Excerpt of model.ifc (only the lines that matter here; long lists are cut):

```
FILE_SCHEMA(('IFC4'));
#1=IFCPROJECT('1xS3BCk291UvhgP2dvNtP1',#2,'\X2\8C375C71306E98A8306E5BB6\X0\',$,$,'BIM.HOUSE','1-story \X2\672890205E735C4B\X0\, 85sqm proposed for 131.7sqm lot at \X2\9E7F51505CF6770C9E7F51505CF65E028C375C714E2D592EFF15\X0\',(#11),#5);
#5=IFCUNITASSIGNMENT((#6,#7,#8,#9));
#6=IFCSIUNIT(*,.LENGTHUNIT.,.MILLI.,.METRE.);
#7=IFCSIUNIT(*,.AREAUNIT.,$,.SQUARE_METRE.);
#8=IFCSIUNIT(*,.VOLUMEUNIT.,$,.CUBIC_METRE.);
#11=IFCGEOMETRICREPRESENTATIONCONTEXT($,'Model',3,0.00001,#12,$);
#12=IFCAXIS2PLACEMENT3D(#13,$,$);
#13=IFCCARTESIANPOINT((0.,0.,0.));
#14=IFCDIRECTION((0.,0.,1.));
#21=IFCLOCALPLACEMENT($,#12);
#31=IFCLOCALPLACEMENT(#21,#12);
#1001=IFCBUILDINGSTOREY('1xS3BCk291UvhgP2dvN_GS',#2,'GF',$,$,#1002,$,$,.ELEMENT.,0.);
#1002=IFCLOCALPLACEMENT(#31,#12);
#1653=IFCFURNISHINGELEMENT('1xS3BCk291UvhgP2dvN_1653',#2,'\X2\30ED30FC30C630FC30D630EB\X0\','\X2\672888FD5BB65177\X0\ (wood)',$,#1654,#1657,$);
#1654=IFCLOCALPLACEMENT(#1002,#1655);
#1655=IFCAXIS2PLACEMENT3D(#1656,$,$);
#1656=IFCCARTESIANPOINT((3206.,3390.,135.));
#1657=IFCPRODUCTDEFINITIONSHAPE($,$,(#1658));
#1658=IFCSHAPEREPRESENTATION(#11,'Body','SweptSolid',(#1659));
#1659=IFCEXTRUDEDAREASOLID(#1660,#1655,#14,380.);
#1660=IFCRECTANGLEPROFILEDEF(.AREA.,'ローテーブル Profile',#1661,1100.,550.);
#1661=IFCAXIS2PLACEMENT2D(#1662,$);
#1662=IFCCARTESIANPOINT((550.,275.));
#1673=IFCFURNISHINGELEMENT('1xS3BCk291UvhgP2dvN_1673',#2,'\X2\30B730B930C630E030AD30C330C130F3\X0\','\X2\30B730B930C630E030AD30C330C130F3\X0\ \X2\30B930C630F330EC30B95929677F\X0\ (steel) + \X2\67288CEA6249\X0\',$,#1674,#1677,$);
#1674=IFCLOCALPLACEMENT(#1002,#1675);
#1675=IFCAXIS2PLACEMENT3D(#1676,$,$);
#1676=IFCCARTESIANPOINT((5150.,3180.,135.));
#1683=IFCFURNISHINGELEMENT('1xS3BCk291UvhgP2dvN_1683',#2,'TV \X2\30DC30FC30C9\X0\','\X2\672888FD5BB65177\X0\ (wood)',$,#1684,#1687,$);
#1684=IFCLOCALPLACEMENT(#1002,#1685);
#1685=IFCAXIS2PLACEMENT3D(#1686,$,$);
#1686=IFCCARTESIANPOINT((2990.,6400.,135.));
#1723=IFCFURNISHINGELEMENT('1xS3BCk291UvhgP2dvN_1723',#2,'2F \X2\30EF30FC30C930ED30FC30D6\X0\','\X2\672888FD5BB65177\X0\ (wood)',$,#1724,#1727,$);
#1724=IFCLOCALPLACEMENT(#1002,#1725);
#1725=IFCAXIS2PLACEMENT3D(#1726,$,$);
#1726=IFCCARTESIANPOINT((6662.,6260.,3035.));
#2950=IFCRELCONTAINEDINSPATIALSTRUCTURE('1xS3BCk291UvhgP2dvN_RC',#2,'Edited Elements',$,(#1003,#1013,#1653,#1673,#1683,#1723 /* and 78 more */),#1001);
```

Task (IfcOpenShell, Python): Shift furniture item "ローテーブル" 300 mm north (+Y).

```python
import ifcopenshell
import ifcopenshell.api.geometry
import ifcopenshell.util.placement
import ifcopenshell.util.unit

model = ifcopenshell.open("model.ifc")
unit_scale = ifcopenshell.util.unit.calculate_unit_scale(model)

item = model.by_id(1653)
matrix = ifcopenshell.util.placement.get_local_placement(item.ObjectPlacement)
matrix[1, 3] += 0.3 / unit_scale
ifcopenshell.api.geometry.edit_object_placement(model, product=item, matrix=matrix, is_si=False)

print(ifcopenshell.util.placement.get_local_placement(item.ObjectPlacement).round(3) + 0.0)

model.write("model-out.ifc")
```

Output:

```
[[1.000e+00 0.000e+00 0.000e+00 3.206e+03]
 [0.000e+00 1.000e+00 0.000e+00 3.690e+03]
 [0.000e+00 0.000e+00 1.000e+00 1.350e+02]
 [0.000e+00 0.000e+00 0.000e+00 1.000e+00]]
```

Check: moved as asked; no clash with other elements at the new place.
